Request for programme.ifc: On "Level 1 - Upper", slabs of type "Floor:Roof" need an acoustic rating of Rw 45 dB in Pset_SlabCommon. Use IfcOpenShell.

First a look at what the model holds.

```python
import ifcopenshell
import ifcopenshell.util.element

model = ifcopenshell.open("programme.ifc")
print(model.schema)
storey = next(s for s in model.by_type("IfcBuildingStorey") if s.Name == "Level 1 - Upper")
slabs = [e for e in ifcopenshell.util.element.get_decomposition(storey) if e.is_a("IfcSlab")]
seen = {}
for e in slabs:
    element_type = ifcopenshell.util.element.get_type(e)
    key = (element_type.Name if element_type != e and element_type else None, ifcopenshell.util.element.get_pset(e, "Pset_SlabCommon", "AcousticRating"))
    seen[key] = seen.get(key, 0) + 1
for (name, value), count in sorted(seen.items(), key=str):
    print(count, "x", name, "|", value)
```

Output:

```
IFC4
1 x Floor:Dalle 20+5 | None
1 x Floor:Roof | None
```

```python
import ifcopenshell
import ifcopenshell.api.pset
import ifcopenshell.util.element

model = ifcopenshell.open("programme.ifc")

storey = next(s for s in model.by_type("IfcBuildingStorey") if s.Name == "Level 1 - Upper")
slabs = [e for e in ifcopenshell.util.element.get_decomposition(storey) if e.is_a("IfcSlab")]

count = 0
for e in slabs:
    element_type = ifcopenshell.util.element.get_type(e)
    if element_type in (None, e) or element_type.Name != "Floor:Roof":
        continue
    # add_pset returns the element's existing set when there is one.
    pset = ifcopenshell.api.pset.add_pset(model, product=e, name="Pset_SlabCommon")
    ifcopenshell.api.pset.edit_pset(model, pset=pset, properties={"AcousticRating": "Rw 45 dB"})
    count += 1

print(count, "slabs updated")

model.write("programme_v2.ifc")
```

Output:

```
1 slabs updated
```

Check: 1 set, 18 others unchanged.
